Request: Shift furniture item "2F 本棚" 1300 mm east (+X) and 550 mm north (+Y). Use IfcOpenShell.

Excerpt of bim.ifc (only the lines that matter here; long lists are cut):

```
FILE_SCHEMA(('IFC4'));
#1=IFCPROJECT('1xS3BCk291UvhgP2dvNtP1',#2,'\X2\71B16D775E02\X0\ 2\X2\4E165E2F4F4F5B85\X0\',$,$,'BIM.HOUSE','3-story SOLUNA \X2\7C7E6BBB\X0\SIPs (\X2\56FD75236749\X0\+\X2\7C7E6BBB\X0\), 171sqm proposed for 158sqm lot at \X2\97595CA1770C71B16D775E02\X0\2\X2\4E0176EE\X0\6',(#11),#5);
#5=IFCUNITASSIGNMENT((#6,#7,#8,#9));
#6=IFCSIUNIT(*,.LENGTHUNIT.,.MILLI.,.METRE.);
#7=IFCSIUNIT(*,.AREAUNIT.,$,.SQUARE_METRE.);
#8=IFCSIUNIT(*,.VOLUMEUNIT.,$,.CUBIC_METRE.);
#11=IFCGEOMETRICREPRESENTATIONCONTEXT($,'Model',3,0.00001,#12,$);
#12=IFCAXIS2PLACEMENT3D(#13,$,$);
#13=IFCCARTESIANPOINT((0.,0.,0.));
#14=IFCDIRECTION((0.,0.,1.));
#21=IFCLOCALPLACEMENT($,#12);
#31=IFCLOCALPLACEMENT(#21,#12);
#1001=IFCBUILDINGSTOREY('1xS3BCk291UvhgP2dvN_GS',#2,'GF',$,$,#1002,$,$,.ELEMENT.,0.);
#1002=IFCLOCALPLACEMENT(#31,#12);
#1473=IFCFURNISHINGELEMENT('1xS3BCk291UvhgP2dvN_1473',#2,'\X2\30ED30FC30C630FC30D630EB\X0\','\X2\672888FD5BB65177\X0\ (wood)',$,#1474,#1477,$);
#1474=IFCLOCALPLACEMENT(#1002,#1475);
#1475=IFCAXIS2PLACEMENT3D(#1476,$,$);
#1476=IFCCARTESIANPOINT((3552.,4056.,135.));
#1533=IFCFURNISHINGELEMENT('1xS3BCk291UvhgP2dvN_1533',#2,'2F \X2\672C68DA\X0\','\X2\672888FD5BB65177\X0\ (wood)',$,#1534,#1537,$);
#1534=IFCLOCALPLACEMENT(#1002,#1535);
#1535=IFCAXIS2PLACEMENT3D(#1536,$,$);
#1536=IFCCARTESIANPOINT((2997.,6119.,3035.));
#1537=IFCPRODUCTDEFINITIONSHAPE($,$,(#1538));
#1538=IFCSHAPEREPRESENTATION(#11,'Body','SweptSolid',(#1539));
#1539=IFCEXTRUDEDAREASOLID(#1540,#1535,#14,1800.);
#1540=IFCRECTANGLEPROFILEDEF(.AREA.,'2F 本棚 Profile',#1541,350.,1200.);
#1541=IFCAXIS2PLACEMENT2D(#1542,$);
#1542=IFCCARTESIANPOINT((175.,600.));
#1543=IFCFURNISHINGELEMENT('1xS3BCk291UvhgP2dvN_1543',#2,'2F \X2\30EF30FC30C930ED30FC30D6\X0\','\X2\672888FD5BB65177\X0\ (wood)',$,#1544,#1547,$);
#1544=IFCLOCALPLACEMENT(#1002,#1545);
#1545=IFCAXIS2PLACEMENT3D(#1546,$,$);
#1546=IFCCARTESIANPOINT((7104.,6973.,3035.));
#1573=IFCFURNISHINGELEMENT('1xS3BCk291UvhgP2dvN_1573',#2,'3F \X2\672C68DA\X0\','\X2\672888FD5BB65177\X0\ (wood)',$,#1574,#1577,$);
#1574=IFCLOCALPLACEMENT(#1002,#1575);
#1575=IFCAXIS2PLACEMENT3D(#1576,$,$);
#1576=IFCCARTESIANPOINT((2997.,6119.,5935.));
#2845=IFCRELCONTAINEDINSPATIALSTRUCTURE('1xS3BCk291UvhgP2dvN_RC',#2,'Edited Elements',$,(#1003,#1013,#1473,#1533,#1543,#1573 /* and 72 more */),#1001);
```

```python
import ifcopenshell
import ifcopenshell.api.geometry
import ifcopenshell.util.placement

model = ifcopenshell.open("bim.ifc")

item = model.by_id(1533)
matrix = ifcopenshell.util.placement.get_local_placement(item.ObjectPlacement)
matrix[0, 3] += 1300.0
matrix[1, 3] += 550.0
ifcopenshell.api.geometry.edit_object_placement(model, product=item, matrix=matrix, is_si=False)

print(ifcopenshell.util.placement.get_local_placement(item.ObjectPlacement).round(3) + 0.0)

model.write("bim_updated.ifc")
```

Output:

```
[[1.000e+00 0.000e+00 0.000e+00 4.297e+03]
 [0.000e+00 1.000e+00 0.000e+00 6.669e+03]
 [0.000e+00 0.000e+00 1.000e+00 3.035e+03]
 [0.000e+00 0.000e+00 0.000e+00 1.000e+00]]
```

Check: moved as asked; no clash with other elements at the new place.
